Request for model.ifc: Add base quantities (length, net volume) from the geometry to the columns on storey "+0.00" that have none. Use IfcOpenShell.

First a look at what the model holds.

```python
import ifcopenshell
import ifcopenshell.util.element
import ifcopenshell.util.unit

model = ifcopenshell.open("model.ifc")
print(model.schema)
for unit_type in ("LENGTHUNIT", "AREAUNIT", "VOLUMEUNIT"):
    print(unit_type, ifcopenshell.util.unit.calculate_unit_scale(model, unit_type))
storey = next(s for s in model.by_type("IfcBuildingStorey") if s.Name == "+0.00")
columns = [e for e in ifcopenshell.util.element.get_decomposition(storey) if e.is_a("IfcColumn")]
for e in sorted(columns, key=lambda e: e.id()):
    print(e.id(), e.is_a(), e.Name, list(ifcopenshell.util.element.get_psets(e, qtos_only=True)), sep=" | ")
```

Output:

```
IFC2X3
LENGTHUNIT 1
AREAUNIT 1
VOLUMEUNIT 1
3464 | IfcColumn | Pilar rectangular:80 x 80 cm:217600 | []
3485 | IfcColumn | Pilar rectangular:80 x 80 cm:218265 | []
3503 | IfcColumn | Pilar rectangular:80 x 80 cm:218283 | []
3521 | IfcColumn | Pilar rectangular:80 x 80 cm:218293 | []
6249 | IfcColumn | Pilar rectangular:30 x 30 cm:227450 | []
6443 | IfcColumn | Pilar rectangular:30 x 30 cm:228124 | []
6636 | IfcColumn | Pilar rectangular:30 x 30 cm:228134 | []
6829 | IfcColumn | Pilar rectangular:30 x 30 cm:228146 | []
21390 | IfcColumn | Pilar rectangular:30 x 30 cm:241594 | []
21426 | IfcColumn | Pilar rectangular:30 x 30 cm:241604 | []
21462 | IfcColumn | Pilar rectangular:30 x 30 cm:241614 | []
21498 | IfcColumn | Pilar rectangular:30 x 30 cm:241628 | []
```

```python
import ifcopenshell
import ifcopenshell.api.pset
import ifcopenshell.geom
import ifcopenshell.util.element
import ifcopenshell.util.shape
import ifcopenshell.util.unit

model = ifcopenshell.open("model.ifc")
unit_scale = ifcopenshell.util.unit.calculate_unit_scale(model)
volume_scale = ifcopenshell.util.unit.calculate_unit_scale(model, "VOLUMEUNIT")
settings = ifcopenshell.geom.settings()

storey = next(s for s in model.by_type("IfcBuildingStorey") if s.Name == "+0.00")
columns = [e for e in ifcopenshell.util.element.get_decomposition(storey) if e.is_a("IfcColumn")]

for e in sorted(columns, key=lambda e: e.id()):
    if ifcopenshell.util.element.get_psets(e, qtos_only=True, should_inherit=False):
        continue
    # Geometry comes back in metres, in the element's own axes.
    shape = ifcopenshell.geom.create_shape(settings, e)
    values = {
        "Length": ifcopenshell.util.shape.get_z(shape.geometry) / unit_scale,
        "NetVolume": ifcopenshell.util.shape.get_volume(shape.geometry) / volume_scale,
    }
    qto = ifcopenshell.api.pset.add_qto(model, product=e, name="BaseQuantities")
    ifcopenshell.api.pset.edit_qto(model, qto=qto, properties=values)
    print(e.id(), {k: round(v, 3) for k, v in values.items()})

model.write("model_edited.ifc")
```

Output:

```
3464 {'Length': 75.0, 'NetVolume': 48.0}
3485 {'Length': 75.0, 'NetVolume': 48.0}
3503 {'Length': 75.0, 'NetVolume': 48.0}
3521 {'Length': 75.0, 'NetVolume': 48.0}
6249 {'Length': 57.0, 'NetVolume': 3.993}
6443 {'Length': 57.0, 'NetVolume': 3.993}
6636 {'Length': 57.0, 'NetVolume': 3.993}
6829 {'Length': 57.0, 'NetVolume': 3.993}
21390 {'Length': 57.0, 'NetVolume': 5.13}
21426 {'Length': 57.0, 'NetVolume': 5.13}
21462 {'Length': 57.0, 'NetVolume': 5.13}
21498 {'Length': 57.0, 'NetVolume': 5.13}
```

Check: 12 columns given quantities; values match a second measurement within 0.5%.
